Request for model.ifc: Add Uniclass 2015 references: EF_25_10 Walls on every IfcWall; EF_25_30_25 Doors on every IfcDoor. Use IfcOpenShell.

First a look at what the model holds.

```python
import ifcopenshell

model = ifcopenshell.open("model.ifc")
print(model.schema)
print("classifications:", [c.Name for c in model.by_type("IfcClassification")])
for ifc_class in ("IfcDoor", "IfcRoof", "IfcStair", "IfcWall", "IfcWindow"):
    print(ifc_class, len(model.by_type(ifc_class)))
```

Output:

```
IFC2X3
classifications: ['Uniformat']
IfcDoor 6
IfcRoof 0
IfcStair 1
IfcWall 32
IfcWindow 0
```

```python
import ifcopenshell
import ifcopenshell.api.classification

model = ifcopenshell.open("model.ifc")

# IFC2X3 requires Source and Edition and has no link from the project to the system.
system = model.create_entity("IfcClassification", Source="NBS", Edition="2015", Name="Uniclass 2015")

codes = {
    "IfcWall": ("EF_25_10", "Walls"),
    "IfcDoor": ("EF_25_30_25", "Doors"),
}
for ifc_class, (code, name) in codes.items():
    products = model.by_type(ifc_class)
    ifcopenshell.api.classification.add_reference(
        model, products=products, classification=system, identification=code, name=name
    )
    print(code, len(products))

model.write("model-out.ifc")
```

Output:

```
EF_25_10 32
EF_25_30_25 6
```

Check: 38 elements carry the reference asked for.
